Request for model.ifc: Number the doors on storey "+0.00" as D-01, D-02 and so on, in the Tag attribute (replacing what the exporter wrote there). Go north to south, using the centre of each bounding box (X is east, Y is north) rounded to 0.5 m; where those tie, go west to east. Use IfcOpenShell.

First a look at what the model holds.

```python
import ifcopenshell
import ifcopenshell.util.element
import ifcopenshell.util.placement

model = ifcopenshell.open("model.ifc")
print(model.schema)
storey = next(s for s in model.by_type("IfcBuildingStorey") if s.Name == "+0.00")
doors = [e for e in ifcopenshell.util.element.get_decomposition(storey) if e.is_a("IfcDoor")]
for e in sorted(doors, key=lambda e: e.id()):
    origin = ifcopenshell.util.placement.get_local_placement(e.ObjectPlacement)[:3, 3]
    print(e.id(), e.Tag, e.Name, origin.round(2) + 0.0, sep=" | ")
```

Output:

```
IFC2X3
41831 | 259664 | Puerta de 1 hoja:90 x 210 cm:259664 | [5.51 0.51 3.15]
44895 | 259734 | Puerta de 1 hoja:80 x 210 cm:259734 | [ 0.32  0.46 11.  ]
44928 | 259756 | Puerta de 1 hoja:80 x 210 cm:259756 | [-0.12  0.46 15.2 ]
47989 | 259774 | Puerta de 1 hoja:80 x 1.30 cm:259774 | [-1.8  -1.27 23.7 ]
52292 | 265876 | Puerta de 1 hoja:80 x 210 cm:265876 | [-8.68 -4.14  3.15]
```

```python
import ifcopenshell
import ifcopenshell.geom
import ifcopenshell.util.element
import ifcopenshell.util.shape

model = ifcopenshell.open("model.ifc")
settings = ifcopenshell.geom.settings()
settings.set("use-world-coords", True)


def centre(element):
    shape = ifcopenshell.geom.create_shape(settings, element)
    return ifcopenshell.util.shape.get_bbox_centroid(shape.geometry)


storey = next(s for s in model.by_type("IfcBuildingStorey") if s.Name == "+0.00")
doors = [e for e in ifcopenshell.util.element.get_decomposition(storey) if e.is_a("IfcDoor")]

# Insertion points can sit at a corner or the storey origin, so sort by the geometry (in metres).
centres = {e: centre(e) for e in doors}
doors.sort(key=lambda e: (-round(centres[e][1] / 0.5), centres[e][0]))

for i, e in enumerate(doors, start=1):
    number = f"D-{i:02d}"
    e.Tag = number
    print(e.id(), number)

model.write("model_v2.ifc")
```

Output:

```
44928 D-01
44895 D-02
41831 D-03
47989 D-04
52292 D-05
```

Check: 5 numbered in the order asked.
